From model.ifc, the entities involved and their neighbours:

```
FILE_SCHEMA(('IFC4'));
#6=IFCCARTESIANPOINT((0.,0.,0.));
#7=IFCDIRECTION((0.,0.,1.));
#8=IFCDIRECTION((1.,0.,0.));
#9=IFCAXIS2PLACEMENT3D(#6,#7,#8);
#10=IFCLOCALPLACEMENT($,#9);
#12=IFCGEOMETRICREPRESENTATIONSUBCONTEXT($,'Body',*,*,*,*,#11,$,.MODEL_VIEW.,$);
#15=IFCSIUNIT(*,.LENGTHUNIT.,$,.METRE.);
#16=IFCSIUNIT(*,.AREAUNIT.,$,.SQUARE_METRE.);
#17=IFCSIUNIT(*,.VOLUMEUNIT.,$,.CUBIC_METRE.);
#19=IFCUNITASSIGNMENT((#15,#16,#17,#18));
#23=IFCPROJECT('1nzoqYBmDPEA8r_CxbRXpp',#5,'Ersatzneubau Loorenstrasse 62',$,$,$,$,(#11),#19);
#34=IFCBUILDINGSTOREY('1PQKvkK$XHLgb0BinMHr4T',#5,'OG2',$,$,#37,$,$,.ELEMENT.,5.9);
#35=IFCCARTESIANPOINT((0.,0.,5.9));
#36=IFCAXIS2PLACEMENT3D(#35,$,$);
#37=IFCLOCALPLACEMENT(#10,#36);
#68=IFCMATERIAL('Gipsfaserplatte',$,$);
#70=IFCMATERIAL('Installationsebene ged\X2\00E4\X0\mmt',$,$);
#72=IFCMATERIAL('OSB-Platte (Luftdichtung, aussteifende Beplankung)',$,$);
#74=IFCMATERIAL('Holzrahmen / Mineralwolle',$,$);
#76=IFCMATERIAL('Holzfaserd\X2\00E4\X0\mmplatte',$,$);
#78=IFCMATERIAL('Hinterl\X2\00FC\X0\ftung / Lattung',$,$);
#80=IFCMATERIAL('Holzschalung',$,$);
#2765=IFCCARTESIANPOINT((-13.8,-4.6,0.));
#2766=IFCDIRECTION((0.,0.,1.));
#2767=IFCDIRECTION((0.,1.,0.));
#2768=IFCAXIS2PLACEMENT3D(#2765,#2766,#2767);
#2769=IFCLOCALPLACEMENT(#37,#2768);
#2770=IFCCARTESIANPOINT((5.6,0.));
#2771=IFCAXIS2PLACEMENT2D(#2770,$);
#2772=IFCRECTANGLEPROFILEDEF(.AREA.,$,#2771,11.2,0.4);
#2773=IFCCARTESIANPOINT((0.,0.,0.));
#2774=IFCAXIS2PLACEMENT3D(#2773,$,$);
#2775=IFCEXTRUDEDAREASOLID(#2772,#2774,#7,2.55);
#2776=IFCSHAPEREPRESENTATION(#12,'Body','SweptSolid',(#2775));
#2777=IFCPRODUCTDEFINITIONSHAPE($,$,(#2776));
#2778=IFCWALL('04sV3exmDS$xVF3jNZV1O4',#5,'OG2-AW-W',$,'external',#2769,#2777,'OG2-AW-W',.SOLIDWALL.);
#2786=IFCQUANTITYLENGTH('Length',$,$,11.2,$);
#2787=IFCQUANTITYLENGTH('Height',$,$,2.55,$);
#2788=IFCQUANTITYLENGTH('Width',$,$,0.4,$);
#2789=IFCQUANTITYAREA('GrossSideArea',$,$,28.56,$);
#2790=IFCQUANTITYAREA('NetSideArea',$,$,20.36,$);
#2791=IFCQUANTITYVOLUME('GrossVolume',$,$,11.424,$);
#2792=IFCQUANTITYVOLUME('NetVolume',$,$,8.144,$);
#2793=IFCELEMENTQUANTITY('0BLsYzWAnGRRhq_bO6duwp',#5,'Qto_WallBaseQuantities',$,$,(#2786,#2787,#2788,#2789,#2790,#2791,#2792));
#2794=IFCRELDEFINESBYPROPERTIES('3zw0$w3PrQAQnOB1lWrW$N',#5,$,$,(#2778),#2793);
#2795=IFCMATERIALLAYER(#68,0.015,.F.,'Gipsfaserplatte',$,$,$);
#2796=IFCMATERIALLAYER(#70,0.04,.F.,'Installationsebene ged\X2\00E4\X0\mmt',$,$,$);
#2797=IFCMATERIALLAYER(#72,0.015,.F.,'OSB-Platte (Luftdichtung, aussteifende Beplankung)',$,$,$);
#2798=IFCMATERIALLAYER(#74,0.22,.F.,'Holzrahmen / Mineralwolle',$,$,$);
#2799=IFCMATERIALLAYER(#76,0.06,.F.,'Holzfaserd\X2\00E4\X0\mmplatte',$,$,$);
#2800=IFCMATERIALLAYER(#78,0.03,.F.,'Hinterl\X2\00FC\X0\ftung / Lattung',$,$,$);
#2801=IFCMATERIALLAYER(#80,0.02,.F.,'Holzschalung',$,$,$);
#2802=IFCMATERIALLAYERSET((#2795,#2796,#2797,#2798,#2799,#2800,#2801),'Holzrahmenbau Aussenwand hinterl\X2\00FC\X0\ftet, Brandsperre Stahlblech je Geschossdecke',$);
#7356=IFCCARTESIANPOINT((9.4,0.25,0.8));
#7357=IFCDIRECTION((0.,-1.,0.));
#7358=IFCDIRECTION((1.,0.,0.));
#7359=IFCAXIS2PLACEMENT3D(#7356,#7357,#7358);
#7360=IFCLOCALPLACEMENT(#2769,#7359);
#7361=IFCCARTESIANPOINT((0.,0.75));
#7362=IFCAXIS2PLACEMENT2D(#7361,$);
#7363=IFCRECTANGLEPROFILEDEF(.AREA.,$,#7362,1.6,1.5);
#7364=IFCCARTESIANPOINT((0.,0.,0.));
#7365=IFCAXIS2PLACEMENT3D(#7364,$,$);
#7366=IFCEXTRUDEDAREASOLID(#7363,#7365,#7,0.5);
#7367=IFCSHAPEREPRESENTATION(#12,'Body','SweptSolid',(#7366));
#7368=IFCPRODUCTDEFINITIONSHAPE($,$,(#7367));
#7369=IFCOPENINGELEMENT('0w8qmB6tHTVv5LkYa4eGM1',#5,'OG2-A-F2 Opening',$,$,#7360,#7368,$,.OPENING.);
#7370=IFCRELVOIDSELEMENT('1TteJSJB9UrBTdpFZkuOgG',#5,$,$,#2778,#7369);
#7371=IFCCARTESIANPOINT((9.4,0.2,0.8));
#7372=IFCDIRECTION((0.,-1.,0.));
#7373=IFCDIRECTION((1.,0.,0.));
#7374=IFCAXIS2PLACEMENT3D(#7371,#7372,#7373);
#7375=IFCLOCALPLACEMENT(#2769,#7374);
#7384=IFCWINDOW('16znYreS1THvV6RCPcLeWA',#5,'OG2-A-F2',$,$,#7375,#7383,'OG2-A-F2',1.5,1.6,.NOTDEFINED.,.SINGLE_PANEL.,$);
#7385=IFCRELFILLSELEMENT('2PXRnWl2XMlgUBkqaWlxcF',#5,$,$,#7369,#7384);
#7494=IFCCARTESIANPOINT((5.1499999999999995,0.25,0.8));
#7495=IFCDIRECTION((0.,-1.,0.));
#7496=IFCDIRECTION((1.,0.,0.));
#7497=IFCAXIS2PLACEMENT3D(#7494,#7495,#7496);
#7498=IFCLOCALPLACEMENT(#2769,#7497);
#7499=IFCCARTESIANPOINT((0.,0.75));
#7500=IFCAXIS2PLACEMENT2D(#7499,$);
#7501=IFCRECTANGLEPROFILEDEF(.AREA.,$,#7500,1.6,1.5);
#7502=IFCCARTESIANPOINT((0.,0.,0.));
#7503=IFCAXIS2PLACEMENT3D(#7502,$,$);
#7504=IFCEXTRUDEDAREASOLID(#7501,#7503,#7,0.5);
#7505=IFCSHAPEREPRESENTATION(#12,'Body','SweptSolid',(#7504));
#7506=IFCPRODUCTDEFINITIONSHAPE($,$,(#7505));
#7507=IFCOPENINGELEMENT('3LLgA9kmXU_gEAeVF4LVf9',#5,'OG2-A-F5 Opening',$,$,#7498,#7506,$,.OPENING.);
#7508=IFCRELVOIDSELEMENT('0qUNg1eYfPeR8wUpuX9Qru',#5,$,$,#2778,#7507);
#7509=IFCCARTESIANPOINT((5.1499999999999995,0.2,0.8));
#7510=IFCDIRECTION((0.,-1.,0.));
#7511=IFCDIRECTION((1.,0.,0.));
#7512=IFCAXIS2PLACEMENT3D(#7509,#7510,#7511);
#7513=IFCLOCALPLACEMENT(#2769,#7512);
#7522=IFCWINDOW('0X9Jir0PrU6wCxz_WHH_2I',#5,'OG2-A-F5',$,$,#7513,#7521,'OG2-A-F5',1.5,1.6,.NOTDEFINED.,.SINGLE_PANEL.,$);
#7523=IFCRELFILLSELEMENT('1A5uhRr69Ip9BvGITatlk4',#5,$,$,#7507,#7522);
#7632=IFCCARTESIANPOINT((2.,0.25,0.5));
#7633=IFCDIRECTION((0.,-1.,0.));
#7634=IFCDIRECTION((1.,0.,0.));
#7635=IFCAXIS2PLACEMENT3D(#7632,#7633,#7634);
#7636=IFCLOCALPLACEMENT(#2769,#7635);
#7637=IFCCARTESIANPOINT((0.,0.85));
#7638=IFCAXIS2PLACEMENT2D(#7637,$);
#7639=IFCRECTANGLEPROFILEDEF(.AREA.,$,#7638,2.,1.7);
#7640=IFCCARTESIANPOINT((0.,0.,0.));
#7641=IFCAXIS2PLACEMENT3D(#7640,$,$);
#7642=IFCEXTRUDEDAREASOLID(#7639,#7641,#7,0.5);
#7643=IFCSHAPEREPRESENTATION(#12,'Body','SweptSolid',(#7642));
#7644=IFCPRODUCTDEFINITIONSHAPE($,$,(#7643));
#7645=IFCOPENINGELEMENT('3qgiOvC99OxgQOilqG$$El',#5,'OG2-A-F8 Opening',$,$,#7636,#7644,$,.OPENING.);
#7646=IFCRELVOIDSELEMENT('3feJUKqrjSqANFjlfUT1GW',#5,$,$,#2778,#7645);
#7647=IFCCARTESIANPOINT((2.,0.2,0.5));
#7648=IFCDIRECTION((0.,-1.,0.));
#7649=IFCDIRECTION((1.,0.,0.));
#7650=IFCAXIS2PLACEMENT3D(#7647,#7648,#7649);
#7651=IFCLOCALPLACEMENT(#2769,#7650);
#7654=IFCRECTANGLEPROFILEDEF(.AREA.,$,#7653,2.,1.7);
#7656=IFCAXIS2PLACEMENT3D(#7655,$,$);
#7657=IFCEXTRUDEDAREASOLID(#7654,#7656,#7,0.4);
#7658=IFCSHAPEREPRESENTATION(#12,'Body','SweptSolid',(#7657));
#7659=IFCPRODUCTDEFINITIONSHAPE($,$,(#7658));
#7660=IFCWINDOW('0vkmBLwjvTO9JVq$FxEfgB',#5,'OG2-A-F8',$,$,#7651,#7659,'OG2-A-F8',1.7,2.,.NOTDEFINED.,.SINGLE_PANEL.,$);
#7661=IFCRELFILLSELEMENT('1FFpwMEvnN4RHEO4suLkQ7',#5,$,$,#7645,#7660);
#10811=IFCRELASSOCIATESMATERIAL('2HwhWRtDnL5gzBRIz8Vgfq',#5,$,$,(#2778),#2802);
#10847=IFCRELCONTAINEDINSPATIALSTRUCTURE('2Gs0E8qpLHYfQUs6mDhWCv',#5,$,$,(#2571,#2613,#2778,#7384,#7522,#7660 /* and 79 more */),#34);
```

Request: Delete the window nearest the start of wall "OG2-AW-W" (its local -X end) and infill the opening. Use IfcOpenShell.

```python
import ifcopenshell
import ifcopenshell.api.feature
import ifcopenshell.api.pset
import ifcopenshell.api.root
import ifcopenshell.geom
import ifcopenshell.util.element
import ifcopenshell.util.shape
import ifcopenshell.util.unit

model = ifcopenshell.open("model.ifc")
area_scale = ifcopenshell.util.unit.calculate_unit_scale(model, "AREAUNIT")
volume_scale = ifcopenshell.util.unit.calculate_unit_scale(model, "VOLUMEUNIT")
settings = ifcopenshell.geom.settings()


def volume(element):
    """Net volume in cubic metres, openings subtracted."""
    shape = ifcopenshell.geom.create_shape(settings, element)
    return ifcopenshell.util.shape.get_volume(shape.geometry)


window = model.by_id(7660)
opening = window.FillsVoids[0].RelatingOpeningElement
wall = opening.VoidsElements[0].RelatingBuildingElement
before = volume(wall)

ifcopenshell.api.root.remove_product(model, product=window)
ifcopenshell.api.feature.remove_feature(model, feature=opening)

after = volume(wall)
thickness = 0.4  # wall thickness in metres

# Update the wall's stored quantities.
qto = model.by_id(ifcopenshell.util.element.get_pset(wall, "Qto_WallBaseQuantities", should_inherit=False)["id"])
ifcopenshell.api.pset.edit_qto(model, qto=qto, properties={
    "NetSideArea": after / thickness / area_scale,
    "NetVolume": after / volume_scale,
})

print(f"wall volume {before:.3f} -> {after:.3f} m3")

model.write("model_edited.ifc")
```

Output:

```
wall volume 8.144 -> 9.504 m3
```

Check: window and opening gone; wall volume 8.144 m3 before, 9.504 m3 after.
